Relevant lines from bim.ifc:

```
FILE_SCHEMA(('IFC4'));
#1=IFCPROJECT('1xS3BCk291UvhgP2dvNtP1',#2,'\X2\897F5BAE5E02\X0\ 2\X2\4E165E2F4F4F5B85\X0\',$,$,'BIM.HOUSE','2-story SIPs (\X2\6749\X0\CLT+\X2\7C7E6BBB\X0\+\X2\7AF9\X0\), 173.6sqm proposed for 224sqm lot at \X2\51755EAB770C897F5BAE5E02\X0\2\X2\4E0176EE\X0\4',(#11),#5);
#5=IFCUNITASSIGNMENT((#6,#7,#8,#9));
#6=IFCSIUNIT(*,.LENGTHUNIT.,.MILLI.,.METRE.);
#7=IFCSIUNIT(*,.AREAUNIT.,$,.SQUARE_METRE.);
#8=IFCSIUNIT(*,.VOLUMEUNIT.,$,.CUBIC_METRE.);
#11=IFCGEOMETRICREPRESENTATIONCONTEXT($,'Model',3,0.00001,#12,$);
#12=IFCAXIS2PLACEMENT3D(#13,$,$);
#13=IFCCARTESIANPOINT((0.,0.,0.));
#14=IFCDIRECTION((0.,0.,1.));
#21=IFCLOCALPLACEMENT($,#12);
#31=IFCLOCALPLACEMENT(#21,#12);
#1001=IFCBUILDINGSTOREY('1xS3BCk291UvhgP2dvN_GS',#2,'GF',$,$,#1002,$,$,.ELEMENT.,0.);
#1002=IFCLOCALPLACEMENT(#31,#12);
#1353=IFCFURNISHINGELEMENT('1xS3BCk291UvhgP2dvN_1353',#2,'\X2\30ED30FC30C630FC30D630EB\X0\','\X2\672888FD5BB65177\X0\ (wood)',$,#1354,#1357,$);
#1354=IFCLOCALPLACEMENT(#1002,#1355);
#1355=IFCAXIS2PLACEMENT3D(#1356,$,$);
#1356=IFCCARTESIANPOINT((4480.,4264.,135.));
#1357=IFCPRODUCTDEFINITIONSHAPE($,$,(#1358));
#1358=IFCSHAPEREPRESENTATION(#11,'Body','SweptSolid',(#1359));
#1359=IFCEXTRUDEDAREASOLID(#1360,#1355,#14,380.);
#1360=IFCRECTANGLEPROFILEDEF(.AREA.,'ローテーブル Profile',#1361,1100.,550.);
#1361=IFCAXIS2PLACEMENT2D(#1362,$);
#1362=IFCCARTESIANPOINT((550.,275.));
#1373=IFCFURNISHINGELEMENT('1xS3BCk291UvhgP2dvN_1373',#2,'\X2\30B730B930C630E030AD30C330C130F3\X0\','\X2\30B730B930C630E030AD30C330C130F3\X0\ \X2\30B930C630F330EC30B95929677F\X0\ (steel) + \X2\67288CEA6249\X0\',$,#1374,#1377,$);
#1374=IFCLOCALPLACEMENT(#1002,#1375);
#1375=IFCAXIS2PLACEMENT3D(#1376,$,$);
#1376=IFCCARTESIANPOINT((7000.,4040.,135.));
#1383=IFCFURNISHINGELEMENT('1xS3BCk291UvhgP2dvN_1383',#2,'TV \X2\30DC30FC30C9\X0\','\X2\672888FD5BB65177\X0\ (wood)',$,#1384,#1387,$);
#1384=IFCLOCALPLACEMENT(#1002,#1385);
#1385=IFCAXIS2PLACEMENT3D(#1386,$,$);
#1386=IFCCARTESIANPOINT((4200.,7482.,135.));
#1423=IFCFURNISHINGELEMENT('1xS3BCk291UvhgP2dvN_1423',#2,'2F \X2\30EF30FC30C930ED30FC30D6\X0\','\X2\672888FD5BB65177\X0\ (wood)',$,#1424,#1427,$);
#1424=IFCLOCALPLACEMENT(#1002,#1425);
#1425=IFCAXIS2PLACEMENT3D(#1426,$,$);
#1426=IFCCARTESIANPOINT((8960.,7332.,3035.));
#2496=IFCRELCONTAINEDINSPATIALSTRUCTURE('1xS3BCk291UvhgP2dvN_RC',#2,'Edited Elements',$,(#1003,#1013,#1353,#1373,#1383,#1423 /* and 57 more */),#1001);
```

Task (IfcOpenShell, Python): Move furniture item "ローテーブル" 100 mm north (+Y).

```python
import ifcopenshell
import ifcopenshell.api.geometry
import ifcopenshell.util.placement
import ifcopenshell.util.unit

model = ifcopenshell.open("bim.ifc")
unit_scale = ifcopenshell.util.unit.calculate_unit_scale(model)

item = model.by_guid("1xS3BCk291UvhgP2dvN_1353")
matrix = ifcopenshell.util.placement.get_local_placement(item.ObjectPlacement)
matrix[1, 3] += 0.1 / unit_scale
ifcopenshell.api.geometry.edit_object_placement(model, product=item, matrix=matrix, is_si=False)

print(ifcopenshell.util.placement.get_local_placement(item.ObjectPlacement).round(3) + 0.0)

model.write("bim_rev.ifc")
```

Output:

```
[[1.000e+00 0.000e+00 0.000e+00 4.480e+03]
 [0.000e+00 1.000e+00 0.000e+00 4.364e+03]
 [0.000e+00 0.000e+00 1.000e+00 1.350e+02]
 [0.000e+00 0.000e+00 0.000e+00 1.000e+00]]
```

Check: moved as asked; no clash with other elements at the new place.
